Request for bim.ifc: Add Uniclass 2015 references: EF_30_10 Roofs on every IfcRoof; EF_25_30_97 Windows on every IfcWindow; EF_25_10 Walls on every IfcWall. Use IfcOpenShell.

First a look at what the model holds.

```python
import ifcopenshell

model = ifcopenshell.open("bim.ifc")
print(model.schema)
print("classifications:", [c.Name for c in model.by_type("IfcClassification")])
for ifc_class in ("IfcDoor", "IfcRoof", "IfcStair", "IfcWall", "IfcWindow"):
    print(ifc_class, len(model.by_type(ifc_class)))
```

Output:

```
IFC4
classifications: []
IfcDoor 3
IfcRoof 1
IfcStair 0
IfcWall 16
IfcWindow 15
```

```python
import ifcopenshell
import ifcopenshell.api.classification

model = ifcopenshell.open("bim.ifc")

system = ifcopenshell.api.classification.add_classification(model, classification="Uniclass 2015")

codes = {
    "IfcRoof": ("EF_30_10", "Roofs"),
    "IfcWindow": ("EF_25_30_97", "Windows"),
    "IfcWall": ("EF_25_10", "Walls"),
}
for ifc_class, (code, name) in codes.items():
    products = model.by_type(ifc_class)
    ifcopenshell.api.classification.add_reference(
        model, products=products, classification=system, identification=code, name=name
    )
    print(code, len(products))

model.write("bim_rev.ifc")
```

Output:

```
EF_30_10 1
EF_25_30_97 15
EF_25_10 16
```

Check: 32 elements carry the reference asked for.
